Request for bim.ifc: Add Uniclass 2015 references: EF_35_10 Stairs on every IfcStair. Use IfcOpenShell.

First a look at what the model holds.

```python
import ifcopenshell

model = ifcopenshell.open("bim.ifc")
print(model.schema)
print("classifications:", [c.Name for c in model.by_type("IfcClassification")])
for ifc_class in ("IfcDoor", "IfcRoof", "IfcStair", "IfcWall", "IfcWindow"):
    print(ifc_class, len(model.by_type(ifc_class)))
```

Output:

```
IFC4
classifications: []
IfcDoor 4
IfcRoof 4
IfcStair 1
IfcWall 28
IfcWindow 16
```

```python
import ifcopenshell
import ifcopenshell.api.classification

model = ifcopenshell.open("bim.ifc")

system = ifcopenshell.api.classification.add_classification(model, classification="Uniclass 2015")

codes = {
    "IfcStair": ("EF_35_10", "Stairs"),
}
for ifc_class, (code, name) in codes.items():
    products = model.by_type(ifc_class)
    ifcopenshell.api.classification.add_reference(
        model, products=products, classification=system, identification=code, name=name
    )
    print(code, len(products))

model.write("bim-out.ifc")
```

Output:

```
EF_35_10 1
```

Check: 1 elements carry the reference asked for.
